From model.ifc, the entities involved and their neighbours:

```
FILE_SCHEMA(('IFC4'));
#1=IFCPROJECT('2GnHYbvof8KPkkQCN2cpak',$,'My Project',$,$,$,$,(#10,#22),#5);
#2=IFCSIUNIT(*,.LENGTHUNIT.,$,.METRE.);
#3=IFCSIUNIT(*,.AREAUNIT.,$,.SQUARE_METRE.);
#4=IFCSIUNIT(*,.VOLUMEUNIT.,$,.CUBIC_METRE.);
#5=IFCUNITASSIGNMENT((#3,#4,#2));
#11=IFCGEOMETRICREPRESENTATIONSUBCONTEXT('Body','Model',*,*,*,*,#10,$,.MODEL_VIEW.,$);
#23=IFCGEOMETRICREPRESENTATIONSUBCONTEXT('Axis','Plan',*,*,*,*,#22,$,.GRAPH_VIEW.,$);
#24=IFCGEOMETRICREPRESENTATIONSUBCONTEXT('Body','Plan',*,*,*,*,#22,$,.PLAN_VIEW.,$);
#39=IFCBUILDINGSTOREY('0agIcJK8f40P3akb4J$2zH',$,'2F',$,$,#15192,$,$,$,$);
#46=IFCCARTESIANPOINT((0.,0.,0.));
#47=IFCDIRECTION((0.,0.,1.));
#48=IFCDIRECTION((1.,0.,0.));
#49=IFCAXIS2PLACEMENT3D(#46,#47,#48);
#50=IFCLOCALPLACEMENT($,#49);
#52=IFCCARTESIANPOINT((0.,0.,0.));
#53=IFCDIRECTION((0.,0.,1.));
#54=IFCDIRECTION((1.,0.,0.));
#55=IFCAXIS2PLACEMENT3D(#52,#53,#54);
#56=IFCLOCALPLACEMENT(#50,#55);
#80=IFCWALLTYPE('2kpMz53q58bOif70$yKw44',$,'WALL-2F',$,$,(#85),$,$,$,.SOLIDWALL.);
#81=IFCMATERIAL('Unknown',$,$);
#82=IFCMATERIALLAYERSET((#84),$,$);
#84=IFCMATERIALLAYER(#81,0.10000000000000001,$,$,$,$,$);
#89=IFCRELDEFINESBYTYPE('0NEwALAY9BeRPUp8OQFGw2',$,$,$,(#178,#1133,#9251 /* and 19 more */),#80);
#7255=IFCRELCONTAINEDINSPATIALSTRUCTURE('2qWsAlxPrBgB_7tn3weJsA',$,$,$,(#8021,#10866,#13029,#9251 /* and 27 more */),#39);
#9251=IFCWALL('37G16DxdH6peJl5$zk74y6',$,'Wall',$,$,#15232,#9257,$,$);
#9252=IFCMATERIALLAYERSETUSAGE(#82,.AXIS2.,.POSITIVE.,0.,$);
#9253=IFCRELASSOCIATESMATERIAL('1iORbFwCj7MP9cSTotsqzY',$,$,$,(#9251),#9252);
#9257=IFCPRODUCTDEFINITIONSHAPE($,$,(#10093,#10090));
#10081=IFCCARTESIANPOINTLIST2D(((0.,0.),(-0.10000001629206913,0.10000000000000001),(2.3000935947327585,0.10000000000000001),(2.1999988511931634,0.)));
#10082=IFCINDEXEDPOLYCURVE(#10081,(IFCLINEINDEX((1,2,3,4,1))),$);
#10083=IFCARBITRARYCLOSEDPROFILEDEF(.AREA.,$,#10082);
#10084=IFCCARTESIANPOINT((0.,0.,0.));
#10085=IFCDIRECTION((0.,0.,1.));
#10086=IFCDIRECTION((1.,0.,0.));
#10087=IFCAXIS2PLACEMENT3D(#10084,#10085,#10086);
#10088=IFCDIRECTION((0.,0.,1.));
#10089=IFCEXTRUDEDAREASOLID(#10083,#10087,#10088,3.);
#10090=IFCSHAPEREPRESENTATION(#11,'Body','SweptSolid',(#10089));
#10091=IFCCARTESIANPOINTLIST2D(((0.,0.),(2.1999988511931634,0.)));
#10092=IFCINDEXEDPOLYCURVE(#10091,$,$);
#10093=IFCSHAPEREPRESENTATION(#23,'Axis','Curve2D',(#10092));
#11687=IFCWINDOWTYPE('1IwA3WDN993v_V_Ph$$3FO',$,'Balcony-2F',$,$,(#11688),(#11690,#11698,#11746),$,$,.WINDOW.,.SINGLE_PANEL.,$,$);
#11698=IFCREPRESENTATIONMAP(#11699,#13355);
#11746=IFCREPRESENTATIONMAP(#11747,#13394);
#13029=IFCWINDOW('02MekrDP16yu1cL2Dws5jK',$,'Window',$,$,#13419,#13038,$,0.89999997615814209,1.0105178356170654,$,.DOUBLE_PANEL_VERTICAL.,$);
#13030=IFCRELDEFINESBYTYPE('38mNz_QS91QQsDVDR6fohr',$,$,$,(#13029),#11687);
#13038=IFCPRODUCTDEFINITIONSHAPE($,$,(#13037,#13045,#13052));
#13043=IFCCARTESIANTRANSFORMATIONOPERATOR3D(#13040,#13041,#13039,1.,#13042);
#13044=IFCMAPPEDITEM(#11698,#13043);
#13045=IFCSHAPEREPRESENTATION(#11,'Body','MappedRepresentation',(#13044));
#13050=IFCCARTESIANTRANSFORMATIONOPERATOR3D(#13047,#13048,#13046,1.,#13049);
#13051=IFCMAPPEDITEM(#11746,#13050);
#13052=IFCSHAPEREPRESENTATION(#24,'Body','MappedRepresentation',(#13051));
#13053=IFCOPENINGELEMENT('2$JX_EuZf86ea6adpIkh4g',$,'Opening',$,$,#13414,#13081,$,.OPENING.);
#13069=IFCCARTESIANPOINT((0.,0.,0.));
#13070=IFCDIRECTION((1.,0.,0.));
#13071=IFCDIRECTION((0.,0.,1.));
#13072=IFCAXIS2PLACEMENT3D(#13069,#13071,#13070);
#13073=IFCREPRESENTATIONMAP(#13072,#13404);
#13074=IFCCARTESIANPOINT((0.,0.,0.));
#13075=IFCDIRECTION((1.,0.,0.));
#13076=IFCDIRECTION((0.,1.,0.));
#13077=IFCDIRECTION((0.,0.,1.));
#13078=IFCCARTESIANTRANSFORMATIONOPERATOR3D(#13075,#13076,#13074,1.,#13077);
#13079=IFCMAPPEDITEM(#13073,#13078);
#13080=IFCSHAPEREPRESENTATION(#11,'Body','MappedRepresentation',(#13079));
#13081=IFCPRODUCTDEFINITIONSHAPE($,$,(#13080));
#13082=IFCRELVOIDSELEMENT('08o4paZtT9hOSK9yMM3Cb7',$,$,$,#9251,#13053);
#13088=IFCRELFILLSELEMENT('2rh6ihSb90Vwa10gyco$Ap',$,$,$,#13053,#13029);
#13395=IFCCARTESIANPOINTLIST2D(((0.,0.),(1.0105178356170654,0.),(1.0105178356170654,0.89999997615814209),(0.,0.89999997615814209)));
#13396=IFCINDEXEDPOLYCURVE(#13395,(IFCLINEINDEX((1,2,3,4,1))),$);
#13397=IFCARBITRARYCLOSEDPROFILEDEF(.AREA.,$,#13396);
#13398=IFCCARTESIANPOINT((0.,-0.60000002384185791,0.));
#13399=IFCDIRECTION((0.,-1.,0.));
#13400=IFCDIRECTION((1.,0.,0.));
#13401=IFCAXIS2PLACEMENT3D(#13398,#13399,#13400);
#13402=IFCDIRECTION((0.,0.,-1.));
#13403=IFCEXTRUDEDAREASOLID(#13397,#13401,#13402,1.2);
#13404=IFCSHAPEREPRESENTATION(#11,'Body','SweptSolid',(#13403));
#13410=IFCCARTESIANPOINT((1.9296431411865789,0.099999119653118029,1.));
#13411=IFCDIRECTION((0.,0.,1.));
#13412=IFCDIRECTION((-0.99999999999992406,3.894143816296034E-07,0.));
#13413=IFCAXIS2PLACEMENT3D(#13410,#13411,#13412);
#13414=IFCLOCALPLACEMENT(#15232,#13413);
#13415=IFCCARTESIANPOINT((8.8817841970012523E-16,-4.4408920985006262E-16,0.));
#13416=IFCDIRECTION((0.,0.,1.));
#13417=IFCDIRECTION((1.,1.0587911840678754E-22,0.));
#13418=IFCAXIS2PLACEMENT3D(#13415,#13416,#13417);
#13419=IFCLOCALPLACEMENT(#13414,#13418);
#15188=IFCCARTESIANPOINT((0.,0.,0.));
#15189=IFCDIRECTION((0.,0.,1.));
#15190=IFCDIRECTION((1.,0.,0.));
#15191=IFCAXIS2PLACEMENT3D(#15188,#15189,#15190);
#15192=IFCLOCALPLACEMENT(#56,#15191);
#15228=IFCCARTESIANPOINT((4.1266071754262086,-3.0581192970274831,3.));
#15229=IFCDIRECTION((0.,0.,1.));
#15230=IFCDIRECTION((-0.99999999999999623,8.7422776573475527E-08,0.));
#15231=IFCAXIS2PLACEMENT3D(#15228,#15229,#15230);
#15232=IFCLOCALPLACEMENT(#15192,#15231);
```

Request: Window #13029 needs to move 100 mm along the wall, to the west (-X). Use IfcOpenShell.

```python
import ifcopenshell
import ifcopenshell.api.geometry
import ifcopenshell.util.placement

model = ifcopenshell.open("model.ifc")

window = model.by_guid("02MekrDP16yu1cL2Dws5jK")
opening = window.FillsVoids[0].RelatingOpeningElement
wall = opening.VoidsElements[0].RelatingBuildingElement

wall_matrix = ifcopenshell.util.placement.get_local_placement(wall.ObjectPlacement)
shift = wall_matrix[:3, 0] * 0.1
before = ifcopenshell.util.placement.get_local_placement(window.ObjectPlacement)[:3, 3].copy()

# The window is placed relative to its opening, so it follows when the opening moves.
matrix = ifcopenshell.util.placement.get_local_placement(opening.ObjectPlacement)
matrix[:3, 3] += shift
ifcopenshell.api.geometry.edit_object_placement(
    model, product=opening, matrix=matrix, is_si=False, should_transform_children=True
)

after = ifcopenshell.util.placement.get_local_placement(window.ObjectPlacement)[:3, 3]
print("window moved by", (after - before).round(3) + 0.0)

model.write("model_rev.ifc")
```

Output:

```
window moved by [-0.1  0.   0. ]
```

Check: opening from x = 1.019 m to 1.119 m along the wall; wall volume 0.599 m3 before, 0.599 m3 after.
